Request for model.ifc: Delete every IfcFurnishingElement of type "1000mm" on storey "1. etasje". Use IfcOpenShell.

First a look at what the model holds.

```python
import ifcopenshell
import ifcopenshell.util.element

model = ifcopenshell.open("model.ifc")
print(model.schema)
storey = next(s for s in model.by_type("IfcBuildingStorey") if s.Name == "1. etasje")
furniture = [e for e in ifcopenshell.util.element.get_decomposition(storey) if e.is_a("IfcFurnishingElement")]
seen = {}
for e in furniture:
    element_type = ifcopenshell.util.element.get_type(e)
    name = element_type.Name if element_type not in (None, e) else None
    seen[name] = seen.get(name, 0) + 1
for name, count in sorted(seen.items(), key=str):
    print(count, "x", name)
```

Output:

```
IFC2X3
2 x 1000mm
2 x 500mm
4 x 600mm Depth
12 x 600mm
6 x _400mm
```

```python
import ifcopenshell
import ifcopenshell.api.root
import ifcopenshell.util.element

model = ifcopenshell.open("model.ifc")

storey = next(s for s in model.by_type("IfcBuildingStorey") if s.Name == "1. etasje")
furniture = [e for e in ifcopenshell.util.element.get_decomposition(storey) if e.is_a("IfcFurnishingElement")]
targets = [e for e in furniture if (t := ifcopenshell.util.element.get_type(e)) not in (None, e) and t.Name == "1000mm"]

for e in targets:
    ifcopenshell.api.root.remove_product(model, product=e)
print(len(targets), "removed")

model.write("model_edited.ifc")
```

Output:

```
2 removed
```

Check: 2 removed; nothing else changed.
